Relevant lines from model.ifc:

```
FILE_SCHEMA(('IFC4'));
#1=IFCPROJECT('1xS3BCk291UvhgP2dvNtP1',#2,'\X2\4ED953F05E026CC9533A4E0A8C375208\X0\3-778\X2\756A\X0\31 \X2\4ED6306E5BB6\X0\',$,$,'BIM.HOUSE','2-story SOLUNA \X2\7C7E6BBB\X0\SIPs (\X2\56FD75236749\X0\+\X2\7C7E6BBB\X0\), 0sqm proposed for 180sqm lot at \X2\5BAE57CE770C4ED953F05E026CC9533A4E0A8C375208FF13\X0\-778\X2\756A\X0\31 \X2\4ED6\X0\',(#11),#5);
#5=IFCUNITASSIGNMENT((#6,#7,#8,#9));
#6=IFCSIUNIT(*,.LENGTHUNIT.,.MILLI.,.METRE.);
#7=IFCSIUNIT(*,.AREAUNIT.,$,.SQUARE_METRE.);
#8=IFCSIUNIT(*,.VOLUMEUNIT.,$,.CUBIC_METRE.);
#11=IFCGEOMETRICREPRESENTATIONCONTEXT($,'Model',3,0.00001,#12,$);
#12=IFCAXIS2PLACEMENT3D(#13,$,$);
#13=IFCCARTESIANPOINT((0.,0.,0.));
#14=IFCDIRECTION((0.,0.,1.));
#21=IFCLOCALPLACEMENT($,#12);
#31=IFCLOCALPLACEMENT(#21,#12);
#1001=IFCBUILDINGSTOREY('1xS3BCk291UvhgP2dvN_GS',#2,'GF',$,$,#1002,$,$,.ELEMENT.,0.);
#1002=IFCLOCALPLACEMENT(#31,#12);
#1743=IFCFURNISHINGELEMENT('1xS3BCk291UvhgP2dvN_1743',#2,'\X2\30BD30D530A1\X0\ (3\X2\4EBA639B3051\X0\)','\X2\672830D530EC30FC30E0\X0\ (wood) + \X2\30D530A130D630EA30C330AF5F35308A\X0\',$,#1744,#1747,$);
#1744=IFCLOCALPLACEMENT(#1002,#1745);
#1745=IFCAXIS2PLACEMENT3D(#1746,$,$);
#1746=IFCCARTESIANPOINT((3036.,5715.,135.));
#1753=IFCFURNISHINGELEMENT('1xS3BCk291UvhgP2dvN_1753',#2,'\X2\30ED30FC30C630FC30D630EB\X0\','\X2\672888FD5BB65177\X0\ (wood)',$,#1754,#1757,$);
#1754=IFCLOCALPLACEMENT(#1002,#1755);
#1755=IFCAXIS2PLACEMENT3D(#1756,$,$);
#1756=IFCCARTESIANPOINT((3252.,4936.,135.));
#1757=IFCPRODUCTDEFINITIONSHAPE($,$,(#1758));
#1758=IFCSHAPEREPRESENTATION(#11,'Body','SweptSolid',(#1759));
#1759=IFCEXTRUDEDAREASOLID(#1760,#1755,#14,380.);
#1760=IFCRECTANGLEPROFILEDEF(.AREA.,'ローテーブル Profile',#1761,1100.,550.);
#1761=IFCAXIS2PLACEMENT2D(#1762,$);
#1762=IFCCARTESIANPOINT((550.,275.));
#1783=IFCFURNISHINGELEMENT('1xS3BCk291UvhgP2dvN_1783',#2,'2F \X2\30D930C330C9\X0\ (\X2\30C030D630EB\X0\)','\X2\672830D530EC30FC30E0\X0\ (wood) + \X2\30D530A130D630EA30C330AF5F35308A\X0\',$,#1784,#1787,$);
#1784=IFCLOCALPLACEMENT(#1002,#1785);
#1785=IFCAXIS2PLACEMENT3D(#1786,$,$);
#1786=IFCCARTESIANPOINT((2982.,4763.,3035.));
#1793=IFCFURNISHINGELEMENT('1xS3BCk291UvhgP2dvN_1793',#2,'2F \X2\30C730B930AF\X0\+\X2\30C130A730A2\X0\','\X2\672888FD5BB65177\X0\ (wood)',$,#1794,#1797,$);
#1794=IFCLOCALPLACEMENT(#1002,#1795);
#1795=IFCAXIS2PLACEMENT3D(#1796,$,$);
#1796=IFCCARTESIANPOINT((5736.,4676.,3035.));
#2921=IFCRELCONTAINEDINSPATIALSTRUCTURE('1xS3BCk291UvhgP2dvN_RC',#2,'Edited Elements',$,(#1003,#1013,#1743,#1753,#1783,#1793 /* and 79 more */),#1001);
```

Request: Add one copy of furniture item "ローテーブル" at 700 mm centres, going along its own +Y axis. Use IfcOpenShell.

```python
import ifcopenshell
import ifcopenshell.api.geometry
import ifcopenshell.api.root
import ifcopenshell.util.element
import ifcopenshell.util.placement
import ifcopenshell.util.unit

model = ifcopenshell.open("model.ifc")
unit_scale = ifcopenshell.util.unit.calculate_unit_scale(model)


def reuse_history(source, copy):
    """copy_class also copies each property set's owner history, people and application; keep the originals."""
    for rel in copy.IsDefinedBy:
        if rel.is_a("IfcRelDefinesByProperties") and (history := rel.RelatingPropertyDefinition.OwnerHistory):
            rel.RelatingPropertyDefinition.OwnerHistory = source.OwnerHistory
            ifcopenshell.util.element.remove_deep2(model, history)


source = model.by_guid("1xS3BCk291UvhgP2dvN_1753")
base = ifcopenshell.util.placement.get_local_placement(source.ObjectPlacement)
step = base[:3, 1] * 0.7 / unit_scale

for i in range(1, 2):
    copy = ifcopenshell.api.root.copy_class(model, product=source)
    copy.Representation = ifcopenshell.util.element.copy_deep(
        model, source.Representation, exclude=["IfcGeometricRepresentationContext", "IfcRepresentationMap"]
    )
    reuse_history(source, copy)
    matrix = base.copy()
    matrix[:3, 3] += i * step
    print("added at", matrix[:3, 3].round(3) + 0.0)
    ifcopenshell.api.geometry.edit_object_placement(model, product=copy, matrix=matrix, is_si=False)

model.write("model_v2.ifc")
```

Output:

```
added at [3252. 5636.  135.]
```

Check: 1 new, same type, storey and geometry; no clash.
